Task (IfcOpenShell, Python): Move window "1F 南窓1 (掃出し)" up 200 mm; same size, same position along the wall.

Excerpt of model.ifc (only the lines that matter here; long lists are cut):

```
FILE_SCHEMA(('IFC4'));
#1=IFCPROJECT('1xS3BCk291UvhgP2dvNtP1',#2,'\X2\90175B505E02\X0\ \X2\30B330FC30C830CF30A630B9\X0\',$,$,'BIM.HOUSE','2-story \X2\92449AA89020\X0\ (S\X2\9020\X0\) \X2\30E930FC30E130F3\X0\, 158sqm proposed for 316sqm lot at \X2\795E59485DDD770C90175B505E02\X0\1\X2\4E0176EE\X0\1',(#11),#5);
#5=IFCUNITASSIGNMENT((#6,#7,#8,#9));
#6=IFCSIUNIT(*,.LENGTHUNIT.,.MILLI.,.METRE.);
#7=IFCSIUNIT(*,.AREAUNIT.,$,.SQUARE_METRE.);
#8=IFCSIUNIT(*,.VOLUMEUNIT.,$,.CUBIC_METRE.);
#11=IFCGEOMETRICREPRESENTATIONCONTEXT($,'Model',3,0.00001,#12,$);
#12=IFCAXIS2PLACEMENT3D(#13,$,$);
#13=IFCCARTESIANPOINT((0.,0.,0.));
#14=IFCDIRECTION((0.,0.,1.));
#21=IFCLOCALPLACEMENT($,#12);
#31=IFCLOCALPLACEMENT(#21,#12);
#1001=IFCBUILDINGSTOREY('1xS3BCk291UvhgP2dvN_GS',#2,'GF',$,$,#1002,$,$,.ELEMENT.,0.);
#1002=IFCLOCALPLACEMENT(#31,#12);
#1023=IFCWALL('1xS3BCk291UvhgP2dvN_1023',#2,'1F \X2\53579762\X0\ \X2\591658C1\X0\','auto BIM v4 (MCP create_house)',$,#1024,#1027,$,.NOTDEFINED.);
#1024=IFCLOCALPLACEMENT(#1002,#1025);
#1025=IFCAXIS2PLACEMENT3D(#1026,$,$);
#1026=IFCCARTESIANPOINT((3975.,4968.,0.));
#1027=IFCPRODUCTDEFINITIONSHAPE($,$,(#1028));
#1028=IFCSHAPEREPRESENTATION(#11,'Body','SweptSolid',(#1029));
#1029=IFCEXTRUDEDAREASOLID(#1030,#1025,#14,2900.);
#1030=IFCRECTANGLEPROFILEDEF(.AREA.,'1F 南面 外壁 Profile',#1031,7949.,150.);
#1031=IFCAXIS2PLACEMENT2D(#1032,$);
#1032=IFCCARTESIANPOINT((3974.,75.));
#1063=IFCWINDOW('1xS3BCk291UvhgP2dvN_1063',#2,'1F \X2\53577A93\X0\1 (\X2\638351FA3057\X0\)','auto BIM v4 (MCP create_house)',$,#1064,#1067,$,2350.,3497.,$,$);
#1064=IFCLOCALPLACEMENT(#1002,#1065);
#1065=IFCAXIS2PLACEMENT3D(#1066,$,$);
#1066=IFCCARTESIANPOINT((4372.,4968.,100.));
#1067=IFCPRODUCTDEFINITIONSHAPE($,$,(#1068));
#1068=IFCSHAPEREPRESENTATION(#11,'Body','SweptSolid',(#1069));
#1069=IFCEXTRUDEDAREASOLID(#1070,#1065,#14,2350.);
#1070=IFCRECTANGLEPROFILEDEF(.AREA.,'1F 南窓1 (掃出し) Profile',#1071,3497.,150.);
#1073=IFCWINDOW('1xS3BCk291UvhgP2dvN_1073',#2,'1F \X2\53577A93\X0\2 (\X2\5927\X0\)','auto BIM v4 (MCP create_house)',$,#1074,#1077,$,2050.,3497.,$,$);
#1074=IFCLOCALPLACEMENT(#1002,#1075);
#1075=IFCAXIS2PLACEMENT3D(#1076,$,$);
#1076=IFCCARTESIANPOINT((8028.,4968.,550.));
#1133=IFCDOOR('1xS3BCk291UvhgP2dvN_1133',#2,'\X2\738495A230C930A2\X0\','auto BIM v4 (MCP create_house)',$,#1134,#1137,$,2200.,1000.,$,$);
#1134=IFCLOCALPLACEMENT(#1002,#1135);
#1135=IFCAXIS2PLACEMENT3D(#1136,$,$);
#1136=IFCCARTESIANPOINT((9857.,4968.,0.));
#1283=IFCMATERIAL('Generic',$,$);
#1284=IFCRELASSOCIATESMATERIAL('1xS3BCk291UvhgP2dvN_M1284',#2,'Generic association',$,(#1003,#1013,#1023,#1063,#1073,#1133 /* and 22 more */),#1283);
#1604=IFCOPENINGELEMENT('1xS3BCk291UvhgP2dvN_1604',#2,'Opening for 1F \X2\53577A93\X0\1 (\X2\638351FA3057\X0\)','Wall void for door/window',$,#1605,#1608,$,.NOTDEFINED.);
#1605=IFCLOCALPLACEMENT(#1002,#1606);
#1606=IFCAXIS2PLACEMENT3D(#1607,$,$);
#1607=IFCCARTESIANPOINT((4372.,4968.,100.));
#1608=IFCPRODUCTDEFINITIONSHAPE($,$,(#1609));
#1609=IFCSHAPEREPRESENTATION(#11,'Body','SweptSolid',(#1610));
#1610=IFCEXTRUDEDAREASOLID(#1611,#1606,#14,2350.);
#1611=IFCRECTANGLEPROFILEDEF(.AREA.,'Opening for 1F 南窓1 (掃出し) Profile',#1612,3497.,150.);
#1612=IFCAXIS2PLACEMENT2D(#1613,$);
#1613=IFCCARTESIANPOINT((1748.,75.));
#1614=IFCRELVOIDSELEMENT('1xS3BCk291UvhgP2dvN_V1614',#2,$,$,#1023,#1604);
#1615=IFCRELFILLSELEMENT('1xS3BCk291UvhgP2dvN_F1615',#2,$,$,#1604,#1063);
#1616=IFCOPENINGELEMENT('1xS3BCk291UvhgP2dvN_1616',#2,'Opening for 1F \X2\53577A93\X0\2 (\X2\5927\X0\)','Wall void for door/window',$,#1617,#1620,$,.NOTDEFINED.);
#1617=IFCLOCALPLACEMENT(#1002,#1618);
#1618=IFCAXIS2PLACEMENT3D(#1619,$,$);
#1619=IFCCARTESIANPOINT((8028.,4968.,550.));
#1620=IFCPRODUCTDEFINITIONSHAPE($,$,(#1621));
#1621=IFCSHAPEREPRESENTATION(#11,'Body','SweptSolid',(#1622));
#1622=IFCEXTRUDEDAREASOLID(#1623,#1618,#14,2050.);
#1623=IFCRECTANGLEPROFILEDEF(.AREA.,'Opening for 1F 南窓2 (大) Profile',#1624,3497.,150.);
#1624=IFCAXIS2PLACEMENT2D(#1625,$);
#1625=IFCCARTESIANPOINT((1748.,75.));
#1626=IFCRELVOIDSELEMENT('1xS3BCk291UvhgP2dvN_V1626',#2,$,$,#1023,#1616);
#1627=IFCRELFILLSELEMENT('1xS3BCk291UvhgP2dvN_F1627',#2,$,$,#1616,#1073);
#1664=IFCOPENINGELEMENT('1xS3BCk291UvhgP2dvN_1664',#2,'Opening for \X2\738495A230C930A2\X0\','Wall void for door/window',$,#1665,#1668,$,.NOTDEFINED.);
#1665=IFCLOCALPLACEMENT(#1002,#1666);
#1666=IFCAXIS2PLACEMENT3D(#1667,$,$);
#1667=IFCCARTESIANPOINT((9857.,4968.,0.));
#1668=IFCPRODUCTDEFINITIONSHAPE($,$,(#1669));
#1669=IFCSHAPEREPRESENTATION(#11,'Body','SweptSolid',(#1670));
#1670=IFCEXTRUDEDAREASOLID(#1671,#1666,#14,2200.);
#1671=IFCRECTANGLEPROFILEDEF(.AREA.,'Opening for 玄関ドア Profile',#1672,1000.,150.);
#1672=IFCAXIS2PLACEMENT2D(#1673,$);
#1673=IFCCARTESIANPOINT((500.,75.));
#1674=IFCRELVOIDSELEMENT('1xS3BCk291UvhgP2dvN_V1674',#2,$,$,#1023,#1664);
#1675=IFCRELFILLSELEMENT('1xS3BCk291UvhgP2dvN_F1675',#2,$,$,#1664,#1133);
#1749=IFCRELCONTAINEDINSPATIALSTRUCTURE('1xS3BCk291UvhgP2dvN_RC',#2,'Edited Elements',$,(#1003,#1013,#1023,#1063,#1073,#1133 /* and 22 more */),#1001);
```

```python
import numpy as np
import ifcopenshell
import ifcopenshell.api.geometry
import ifcopenshell.util.placement
import ifcopenshell.util.unit

model = ifcopenshell.open("model.ifc")
unit_scale = ifcopenshell.util.unit.calculate_unit_scale(model)

window = model.by_guid("1xS3BCk291UvhgP2dvN_1063")
opening = window.FillsVoids[0].RelatingOpeningElement
dz = 200.0

shift = np.array([0.0, 0.0, dz])
# The window is not placed relative to its opening, so move both.
for product in (opening, window):
    matrix = ifcopenshell.util.placement.get_local_placement(product.ObjectPlacement)
    matrix[:3, 3] += shift
    ifcopenshell.api.geometry.edit_object_placement(model, product=product, matrix=matrix, is_si=False)

print(f"moved by {dz * unit_scale:+.3f} m")

model.write("model_v2.ifc")
```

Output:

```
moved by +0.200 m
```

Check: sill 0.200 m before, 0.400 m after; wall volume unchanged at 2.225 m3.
